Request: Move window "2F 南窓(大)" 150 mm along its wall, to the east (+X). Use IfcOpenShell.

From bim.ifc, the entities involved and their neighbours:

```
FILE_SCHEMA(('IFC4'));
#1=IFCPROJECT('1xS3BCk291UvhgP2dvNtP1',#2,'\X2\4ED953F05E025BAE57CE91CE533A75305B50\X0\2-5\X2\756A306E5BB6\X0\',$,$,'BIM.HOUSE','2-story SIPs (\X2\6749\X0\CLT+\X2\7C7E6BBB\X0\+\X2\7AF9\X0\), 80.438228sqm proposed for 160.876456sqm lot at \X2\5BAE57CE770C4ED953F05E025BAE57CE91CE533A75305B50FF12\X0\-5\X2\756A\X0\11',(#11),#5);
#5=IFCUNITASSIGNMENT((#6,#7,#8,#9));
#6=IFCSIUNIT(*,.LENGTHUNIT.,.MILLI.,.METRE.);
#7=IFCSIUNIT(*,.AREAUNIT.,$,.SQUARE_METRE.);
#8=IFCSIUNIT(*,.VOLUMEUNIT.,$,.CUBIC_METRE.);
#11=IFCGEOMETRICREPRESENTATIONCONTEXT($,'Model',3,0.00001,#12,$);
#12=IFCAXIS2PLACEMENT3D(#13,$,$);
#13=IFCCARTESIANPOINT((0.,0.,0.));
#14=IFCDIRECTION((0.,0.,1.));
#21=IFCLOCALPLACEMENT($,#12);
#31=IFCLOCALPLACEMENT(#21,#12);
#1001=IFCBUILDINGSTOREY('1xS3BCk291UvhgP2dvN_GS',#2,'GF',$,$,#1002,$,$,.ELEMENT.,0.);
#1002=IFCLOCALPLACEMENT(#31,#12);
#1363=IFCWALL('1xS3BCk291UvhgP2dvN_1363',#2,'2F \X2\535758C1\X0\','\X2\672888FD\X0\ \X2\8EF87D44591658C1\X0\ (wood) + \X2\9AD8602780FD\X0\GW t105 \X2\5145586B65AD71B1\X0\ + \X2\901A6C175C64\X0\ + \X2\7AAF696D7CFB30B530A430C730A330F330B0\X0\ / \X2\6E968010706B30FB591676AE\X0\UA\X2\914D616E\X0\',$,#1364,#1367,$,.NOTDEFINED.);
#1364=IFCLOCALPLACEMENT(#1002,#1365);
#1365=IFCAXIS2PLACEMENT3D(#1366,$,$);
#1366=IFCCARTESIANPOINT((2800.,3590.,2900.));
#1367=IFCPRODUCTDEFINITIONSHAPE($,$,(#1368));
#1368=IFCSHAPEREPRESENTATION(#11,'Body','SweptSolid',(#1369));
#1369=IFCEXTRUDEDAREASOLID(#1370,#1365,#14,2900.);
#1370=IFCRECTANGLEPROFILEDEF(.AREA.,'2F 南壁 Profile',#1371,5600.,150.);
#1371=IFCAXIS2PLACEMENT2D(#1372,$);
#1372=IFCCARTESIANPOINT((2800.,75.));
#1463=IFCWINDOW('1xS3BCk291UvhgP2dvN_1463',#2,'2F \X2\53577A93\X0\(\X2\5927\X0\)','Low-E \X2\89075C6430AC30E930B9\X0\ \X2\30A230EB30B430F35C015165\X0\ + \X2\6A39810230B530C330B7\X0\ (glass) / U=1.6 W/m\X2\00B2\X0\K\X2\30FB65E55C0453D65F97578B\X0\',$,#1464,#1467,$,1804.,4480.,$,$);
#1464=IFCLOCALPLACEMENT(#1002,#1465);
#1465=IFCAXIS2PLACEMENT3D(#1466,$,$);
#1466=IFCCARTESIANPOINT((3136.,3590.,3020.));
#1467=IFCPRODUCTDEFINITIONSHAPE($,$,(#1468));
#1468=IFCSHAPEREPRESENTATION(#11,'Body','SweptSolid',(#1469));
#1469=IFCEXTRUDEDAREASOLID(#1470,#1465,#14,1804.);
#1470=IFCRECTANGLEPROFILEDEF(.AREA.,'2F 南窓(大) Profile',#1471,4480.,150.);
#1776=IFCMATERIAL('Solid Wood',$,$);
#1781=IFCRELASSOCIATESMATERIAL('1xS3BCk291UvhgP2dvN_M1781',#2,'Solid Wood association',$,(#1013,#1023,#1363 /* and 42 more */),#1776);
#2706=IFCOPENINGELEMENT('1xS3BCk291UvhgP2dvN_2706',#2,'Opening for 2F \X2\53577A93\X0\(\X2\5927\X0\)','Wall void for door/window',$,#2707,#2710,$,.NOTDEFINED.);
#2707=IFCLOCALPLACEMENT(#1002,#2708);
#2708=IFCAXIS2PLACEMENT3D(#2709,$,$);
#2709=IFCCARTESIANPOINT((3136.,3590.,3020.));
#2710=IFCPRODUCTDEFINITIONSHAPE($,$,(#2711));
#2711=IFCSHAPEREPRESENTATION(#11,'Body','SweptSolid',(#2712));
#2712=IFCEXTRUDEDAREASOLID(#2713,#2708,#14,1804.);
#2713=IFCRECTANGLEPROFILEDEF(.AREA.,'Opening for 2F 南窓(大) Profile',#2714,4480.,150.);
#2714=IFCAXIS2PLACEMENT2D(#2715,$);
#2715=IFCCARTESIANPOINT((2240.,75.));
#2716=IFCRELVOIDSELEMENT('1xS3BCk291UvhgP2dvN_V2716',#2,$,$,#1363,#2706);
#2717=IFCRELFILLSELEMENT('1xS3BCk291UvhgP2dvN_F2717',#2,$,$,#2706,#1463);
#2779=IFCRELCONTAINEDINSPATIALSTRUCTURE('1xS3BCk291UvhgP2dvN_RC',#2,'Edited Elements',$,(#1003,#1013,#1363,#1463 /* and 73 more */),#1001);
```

```python
import ifcopenshell
import ifcopenshell.api.geometry
import ifcopenshell.util.placement

model = ifcopenshell.open("bim.ifc")

window = model.by_id(1463)
opening = window.FillsVoids[0].RelatingOpeningElement
wall = opening.VoidsElements[0].RelatingBuildingElement

wall_matrix = ifcopenshell.util.placement.get_local_placement(wall.ObjectPlacement)
shift = wall_matrix[:3, 0] * 150.0
before = ifcopenshell.util.placement.get_local_placement(window.ObjectPlacement)[:3, 3].copy()

# The window is not placed relative to its opening, so move both.
for product in (opening, window):
    matrix = ifcopenshell.util.placement.get_local_placement(product.ObjectPlacement)
    matrix[:3, 3] += shift
    ifcopenshell.api.geometry.edit_object_placement(model, product=product, matrix=matrix, is_si=False)

after = ifcopenshell.util.placement.get_local_placement(window.ObjectPlacement)[:3, 3]
print("window moved by", (after - before).round(3) + 0.0)

model.write("bim-out.ifc")
```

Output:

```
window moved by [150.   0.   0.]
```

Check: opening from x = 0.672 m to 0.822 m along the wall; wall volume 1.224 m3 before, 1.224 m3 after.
